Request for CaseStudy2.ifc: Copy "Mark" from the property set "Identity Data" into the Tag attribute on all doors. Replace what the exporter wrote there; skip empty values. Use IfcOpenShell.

First a look at what the model holds.

```python
import ifcopenshell
import ifcopenshell.util.element

model = ifcopenshell.open("CaseStudy2.ifc")
print(model.schema)
doors = model.by_type("IfcDoor")
print(len(doors), "doors")
for e in doors[:8]:
    source = ifcopenshell.util.element.get_pset(e, "Identity Data", "Mark")
    target = e.Tag
    print(e.id(), repr(source), repr(target), sep=" | ")
```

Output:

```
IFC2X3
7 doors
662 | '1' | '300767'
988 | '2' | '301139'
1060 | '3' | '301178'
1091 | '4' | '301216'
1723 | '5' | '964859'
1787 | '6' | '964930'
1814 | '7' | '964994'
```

```python
import ifcopenshell
import ifcopenshell.util.element

model = ifcopenshell.open("CaseStudy2.ifc")

count = 0
for e in model.by_type("IfcDoor"):
    value = ifcopenshell.util.element.get_pset(e, "Identity Data", "Mark")
    current = e.Tag
    if not value or not value.strip() or current == value:
        continue
    e.Tag = value
    count += 1

print(count, "doors updated")

model.write("CaseStudy2-out.ifc")
```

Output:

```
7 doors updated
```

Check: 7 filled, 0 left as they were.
